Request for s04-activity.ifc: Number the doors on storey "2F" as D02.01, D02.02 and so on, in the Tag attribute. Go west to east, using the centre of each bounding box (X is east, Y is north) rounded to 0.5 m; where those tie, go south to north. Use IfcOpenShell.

First a look at what the model holds.

```python
import ifcopenshell
import ifcopenshell.util.element
import ifcopenshell.util.placement

model = ifcopenshell.open("s04-activity.ifc")
print(model.schema)
storey = next(s for s in model.by_type("IfcBuildingStorey") if s.Name == "2F")
doors = [e for e in ifcopenshell.util.element.get_decomposition(storey) if e.is_a("IfcDoor")]
for e in sorted(doors, key=lambda e: e.id()):
    origin = ifcopenshell.util.placement.get_local_placement(e.ObjectPlacement)[:3, 3]
    print(e.id(), e.Tag, e.Name, origin.round(2) + 0.0, sep=" | ")
```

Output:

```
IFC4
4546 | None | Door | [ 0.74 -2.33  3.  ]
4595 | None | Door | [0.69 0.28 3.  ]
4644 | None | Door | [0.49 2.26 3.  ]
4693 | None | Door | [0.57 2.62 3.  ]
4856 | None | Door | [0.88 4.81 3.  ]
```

```python
import ifcopenshell
import ifcopenshell.geom
import ifcopenshell.util.element
import ifcopenshell.util.shape

model = ifcopenshell.open("s04-activity.ifc")
settings = ifcopenshell.geom.settings()
settings.set("use-world-coords", True)


def centre(element):
    shape = ifcopenshell.geom.create_shape(settings, element)
    return ifcopenshell.util.shape.get_bbox_centroid(shape.geometry)


storey = next(s for s in model.by_type("IfcBuildingStorey") if s.Name == "2F")
doors = [e for e in ifcopenshell.util.element.get_decomposition(storey) if e.is_a("IfcDoor")]

# Insertion points can sit at a corner or the storey origin, so sort by the geometry (in metres).
centres = {e: centre(e) for e in doors}
doors.sort(key=lambda e: (round(centres[e][0] / 0.5), centres[e][1]))

for i, e in enumerate(doors, start=1):
    number = f"D02.{i:02d}"
    e.Tag = number
    print(e.id(), number)

model.write("s04-activity_edited.ifc")
```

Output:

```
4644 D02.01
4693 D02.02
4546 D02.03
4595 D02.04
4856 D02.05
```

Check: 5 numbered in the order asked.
